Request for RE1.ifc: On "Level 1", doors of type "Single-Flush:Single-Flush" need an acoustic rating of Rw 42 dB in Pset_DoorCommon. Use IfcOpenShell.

First a look at what the model holds.

```python
import ifcopenshell
import ifcopenshell.util.element

model = ifcopenshell.open("RE1.ifc")
print(model.schema)
storey = next(s for s in model.by_type("IfcBuildingStorey") if s.Name == "Level 1")
doors = [e for e in ifcopenshell.util.element.get_decomposition(storey) if e.is_a("IfcDoor")]
seen = {}
for e in doors:
    element_type = ifcopenshell.util.element.get_type(e)
    key = (element_type.Name if element_type != e and element_type else None, ifcopenshell.util.element.get_pset(e, "Pset_DoorCommon", "AcousticRating"))
    seen[key] = seen.get(key, 0) + 1
for (name, value), count in sorted(seen.items(), key=str):
    print(count, "x", name, "|", value)
```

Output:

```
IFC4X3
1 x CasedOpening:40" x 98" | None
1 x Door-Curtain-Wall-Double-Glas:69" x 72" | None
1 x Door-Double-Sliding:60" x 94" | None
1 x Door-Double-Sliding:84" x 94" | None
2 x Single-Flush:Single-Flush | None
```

```python
import ifcopenshell
import ifcopenshell.api.pset
import ifcopenshell.util.element

model = ifcopenshell.open("RE1.ifc")

storey = next(s for s in model.by_type("IfcBuildingStorey") if s.Name == "Level 1")
doors = [e for e in ifcopenshell.util.element.get_decomposition(storey) if e.is_a("IfcDoor")]

count = 0
for e in doors:
    element_type = ifcopenshell.util.element.get_type(e)
    if element_type in (None, e) or element_type.Name != "Single-Flush:Single-Flush":
        continue
    # add_pset returns the element's existing set when there is one.
    pset = ifcopenshell.api.pset.add_pset(model, product=e, name="Pset_DoorCommon")
    ifcopenshell.api.pset.edit_pset(model, pset=pset, properties={"AcousticRating": "Rw 42 dB"})
    count += 1

print(count, "doors updated")

model.write("RE1_edited.ifc")
```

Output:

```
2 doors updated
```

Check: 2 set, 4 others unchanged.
